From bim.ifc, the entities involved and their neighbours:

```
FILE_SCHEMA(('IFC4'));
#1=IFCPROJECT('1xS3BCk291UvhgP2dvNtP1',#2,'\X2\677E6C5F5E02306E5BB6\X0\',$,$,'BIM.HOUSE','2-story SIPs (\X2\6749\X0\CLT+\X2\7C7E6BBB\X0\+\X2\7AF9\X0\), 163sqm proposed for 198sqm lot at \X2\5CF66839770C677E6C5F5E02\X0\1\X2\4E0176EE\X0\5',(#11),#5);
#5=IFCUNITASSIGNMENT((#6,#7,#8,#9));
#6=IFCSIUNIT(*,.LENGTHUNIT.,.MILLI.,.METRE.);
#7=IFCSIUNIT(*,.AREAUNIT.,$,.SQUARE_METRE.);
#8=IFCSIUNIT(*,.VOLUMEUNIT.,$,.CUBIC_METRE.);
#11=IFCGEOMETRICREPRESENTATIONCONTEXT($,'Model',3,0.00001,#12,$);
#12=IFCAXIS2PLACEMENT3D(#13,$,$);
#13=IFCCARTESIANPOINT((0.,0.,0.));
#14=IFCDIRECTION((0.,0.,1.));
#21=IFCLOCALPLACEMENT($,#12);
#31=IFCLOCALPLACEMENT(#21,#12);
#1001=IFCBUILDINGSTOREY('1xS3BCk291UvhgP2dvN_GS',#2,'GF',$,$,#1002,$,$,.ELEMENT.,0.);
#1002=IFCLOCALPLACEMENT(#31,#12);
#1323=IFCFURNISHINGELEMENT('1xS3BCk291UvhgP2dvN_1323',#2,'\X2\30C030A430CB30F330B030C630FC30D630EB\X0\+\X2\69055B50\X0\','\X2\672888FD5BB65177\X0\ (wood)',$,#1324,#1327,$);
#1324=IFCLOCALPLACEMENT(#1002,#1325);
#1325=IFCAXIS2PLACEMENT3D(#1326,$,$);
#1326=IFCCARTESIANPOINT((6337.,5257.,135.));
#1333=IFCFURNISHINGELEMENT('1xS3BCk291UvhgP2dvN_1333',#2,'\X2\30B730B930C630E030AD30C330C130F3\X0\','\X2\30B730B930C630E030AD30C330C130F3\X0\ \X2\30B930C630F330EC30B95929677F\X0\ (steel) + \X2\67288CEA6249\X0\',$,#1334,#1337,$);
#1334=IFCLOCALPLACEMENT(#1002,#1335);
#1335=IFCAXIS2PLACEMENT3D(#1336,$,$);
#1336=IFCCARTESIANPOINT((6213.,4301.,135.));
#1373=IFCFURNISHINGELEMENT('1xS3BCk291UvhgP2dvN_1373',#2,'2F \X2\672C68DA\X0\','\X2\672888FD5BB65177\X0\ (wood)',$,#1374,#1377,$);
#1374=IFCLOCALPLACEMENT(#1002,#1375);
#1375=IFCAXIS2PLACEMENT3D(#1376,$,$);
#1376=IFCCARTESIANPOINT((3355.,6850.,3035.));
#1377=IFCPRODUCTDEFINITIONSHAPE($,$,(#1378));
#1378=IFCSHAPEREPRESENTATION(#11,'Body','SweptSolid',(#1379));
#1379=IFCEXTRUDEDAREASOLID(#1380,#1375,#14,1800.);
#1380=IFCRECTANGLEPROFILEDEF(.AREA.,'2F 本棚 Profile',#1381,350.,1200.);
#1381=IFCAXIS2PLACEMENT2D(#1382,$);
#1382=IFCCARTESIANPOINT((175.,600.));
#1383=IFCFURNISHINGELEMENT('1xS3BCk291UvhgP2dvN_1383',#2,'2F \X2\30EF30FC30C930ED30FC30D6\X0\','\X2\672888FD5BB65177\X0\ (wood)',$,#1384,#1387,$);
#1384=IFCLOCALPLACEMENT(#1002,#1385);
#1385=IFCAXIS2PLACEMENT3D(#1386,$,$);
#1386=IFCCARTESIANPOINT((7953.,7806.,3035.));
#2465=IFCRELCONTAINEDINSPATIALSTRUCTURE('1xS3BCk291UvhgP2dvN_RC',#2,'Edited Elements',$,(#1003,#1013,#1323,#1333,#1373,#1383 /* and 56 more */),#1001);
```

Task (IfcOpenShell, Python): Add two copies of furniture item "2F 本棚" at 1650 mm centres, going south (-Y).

```python
import numpy as np
import ifcopenshell
import ifcopenshell.api.geometry
import ifcopenshell.api.root
import ifcopenshell.util.element
import ifcopenshell.util.placement
import ifcopenshell.util.unit

model = ifcopenshell.open("bim.ifc")
unit_scale = ifcopenshell.util.unit.calculate_unit_scale(model)


def reuse_history(source, copy):
    """copy_class also copies each property set's owner history, people and application; keep the originals."""
    for rel in copy.IsDefinedBy:
        if rel.is_a("IfcRelDefinesByProperties") and (history := rel.RelatingPropertyDefinition.OwnerHistory):
            rel.RelatingPropertyDefinition.OwnerHistory = source.OwnerHistory
            ifcopenshell.util.element.remove_deep2(model, history)


source = model.by_id(1373)
base = ifcopenshell.util.placement.get_local_placement(source.ObjectPlacement)
step = np.array([0.0, -1.0, 0.0]) * 1.65 / unit_scale

for i in range(1, 3):
    copy = ifcopenshell.api.root.copy_class(model, product=source)
    copy.Representation = ifcopenshell.util.element.copy_deep(
        model, source.Representation, exclude=["IfcGeometricRepresentationContext", "IfcRepresentationMap"]
    )
    reuse_history(source, copy)
    matrix = base.copy()
    matrix[:3, 3] += i * step
    print("added at", matrix[:3, 3].round(3) + 0.0)
    ifcopenshell.api.geometry.edit_object_placement(model, product=copy, matrix=matrix, is_si=False)

model.write("bim_v2.ifc")
```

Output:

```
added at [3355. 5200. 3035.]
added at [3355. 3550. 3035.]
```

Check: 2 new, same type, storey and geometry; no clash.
